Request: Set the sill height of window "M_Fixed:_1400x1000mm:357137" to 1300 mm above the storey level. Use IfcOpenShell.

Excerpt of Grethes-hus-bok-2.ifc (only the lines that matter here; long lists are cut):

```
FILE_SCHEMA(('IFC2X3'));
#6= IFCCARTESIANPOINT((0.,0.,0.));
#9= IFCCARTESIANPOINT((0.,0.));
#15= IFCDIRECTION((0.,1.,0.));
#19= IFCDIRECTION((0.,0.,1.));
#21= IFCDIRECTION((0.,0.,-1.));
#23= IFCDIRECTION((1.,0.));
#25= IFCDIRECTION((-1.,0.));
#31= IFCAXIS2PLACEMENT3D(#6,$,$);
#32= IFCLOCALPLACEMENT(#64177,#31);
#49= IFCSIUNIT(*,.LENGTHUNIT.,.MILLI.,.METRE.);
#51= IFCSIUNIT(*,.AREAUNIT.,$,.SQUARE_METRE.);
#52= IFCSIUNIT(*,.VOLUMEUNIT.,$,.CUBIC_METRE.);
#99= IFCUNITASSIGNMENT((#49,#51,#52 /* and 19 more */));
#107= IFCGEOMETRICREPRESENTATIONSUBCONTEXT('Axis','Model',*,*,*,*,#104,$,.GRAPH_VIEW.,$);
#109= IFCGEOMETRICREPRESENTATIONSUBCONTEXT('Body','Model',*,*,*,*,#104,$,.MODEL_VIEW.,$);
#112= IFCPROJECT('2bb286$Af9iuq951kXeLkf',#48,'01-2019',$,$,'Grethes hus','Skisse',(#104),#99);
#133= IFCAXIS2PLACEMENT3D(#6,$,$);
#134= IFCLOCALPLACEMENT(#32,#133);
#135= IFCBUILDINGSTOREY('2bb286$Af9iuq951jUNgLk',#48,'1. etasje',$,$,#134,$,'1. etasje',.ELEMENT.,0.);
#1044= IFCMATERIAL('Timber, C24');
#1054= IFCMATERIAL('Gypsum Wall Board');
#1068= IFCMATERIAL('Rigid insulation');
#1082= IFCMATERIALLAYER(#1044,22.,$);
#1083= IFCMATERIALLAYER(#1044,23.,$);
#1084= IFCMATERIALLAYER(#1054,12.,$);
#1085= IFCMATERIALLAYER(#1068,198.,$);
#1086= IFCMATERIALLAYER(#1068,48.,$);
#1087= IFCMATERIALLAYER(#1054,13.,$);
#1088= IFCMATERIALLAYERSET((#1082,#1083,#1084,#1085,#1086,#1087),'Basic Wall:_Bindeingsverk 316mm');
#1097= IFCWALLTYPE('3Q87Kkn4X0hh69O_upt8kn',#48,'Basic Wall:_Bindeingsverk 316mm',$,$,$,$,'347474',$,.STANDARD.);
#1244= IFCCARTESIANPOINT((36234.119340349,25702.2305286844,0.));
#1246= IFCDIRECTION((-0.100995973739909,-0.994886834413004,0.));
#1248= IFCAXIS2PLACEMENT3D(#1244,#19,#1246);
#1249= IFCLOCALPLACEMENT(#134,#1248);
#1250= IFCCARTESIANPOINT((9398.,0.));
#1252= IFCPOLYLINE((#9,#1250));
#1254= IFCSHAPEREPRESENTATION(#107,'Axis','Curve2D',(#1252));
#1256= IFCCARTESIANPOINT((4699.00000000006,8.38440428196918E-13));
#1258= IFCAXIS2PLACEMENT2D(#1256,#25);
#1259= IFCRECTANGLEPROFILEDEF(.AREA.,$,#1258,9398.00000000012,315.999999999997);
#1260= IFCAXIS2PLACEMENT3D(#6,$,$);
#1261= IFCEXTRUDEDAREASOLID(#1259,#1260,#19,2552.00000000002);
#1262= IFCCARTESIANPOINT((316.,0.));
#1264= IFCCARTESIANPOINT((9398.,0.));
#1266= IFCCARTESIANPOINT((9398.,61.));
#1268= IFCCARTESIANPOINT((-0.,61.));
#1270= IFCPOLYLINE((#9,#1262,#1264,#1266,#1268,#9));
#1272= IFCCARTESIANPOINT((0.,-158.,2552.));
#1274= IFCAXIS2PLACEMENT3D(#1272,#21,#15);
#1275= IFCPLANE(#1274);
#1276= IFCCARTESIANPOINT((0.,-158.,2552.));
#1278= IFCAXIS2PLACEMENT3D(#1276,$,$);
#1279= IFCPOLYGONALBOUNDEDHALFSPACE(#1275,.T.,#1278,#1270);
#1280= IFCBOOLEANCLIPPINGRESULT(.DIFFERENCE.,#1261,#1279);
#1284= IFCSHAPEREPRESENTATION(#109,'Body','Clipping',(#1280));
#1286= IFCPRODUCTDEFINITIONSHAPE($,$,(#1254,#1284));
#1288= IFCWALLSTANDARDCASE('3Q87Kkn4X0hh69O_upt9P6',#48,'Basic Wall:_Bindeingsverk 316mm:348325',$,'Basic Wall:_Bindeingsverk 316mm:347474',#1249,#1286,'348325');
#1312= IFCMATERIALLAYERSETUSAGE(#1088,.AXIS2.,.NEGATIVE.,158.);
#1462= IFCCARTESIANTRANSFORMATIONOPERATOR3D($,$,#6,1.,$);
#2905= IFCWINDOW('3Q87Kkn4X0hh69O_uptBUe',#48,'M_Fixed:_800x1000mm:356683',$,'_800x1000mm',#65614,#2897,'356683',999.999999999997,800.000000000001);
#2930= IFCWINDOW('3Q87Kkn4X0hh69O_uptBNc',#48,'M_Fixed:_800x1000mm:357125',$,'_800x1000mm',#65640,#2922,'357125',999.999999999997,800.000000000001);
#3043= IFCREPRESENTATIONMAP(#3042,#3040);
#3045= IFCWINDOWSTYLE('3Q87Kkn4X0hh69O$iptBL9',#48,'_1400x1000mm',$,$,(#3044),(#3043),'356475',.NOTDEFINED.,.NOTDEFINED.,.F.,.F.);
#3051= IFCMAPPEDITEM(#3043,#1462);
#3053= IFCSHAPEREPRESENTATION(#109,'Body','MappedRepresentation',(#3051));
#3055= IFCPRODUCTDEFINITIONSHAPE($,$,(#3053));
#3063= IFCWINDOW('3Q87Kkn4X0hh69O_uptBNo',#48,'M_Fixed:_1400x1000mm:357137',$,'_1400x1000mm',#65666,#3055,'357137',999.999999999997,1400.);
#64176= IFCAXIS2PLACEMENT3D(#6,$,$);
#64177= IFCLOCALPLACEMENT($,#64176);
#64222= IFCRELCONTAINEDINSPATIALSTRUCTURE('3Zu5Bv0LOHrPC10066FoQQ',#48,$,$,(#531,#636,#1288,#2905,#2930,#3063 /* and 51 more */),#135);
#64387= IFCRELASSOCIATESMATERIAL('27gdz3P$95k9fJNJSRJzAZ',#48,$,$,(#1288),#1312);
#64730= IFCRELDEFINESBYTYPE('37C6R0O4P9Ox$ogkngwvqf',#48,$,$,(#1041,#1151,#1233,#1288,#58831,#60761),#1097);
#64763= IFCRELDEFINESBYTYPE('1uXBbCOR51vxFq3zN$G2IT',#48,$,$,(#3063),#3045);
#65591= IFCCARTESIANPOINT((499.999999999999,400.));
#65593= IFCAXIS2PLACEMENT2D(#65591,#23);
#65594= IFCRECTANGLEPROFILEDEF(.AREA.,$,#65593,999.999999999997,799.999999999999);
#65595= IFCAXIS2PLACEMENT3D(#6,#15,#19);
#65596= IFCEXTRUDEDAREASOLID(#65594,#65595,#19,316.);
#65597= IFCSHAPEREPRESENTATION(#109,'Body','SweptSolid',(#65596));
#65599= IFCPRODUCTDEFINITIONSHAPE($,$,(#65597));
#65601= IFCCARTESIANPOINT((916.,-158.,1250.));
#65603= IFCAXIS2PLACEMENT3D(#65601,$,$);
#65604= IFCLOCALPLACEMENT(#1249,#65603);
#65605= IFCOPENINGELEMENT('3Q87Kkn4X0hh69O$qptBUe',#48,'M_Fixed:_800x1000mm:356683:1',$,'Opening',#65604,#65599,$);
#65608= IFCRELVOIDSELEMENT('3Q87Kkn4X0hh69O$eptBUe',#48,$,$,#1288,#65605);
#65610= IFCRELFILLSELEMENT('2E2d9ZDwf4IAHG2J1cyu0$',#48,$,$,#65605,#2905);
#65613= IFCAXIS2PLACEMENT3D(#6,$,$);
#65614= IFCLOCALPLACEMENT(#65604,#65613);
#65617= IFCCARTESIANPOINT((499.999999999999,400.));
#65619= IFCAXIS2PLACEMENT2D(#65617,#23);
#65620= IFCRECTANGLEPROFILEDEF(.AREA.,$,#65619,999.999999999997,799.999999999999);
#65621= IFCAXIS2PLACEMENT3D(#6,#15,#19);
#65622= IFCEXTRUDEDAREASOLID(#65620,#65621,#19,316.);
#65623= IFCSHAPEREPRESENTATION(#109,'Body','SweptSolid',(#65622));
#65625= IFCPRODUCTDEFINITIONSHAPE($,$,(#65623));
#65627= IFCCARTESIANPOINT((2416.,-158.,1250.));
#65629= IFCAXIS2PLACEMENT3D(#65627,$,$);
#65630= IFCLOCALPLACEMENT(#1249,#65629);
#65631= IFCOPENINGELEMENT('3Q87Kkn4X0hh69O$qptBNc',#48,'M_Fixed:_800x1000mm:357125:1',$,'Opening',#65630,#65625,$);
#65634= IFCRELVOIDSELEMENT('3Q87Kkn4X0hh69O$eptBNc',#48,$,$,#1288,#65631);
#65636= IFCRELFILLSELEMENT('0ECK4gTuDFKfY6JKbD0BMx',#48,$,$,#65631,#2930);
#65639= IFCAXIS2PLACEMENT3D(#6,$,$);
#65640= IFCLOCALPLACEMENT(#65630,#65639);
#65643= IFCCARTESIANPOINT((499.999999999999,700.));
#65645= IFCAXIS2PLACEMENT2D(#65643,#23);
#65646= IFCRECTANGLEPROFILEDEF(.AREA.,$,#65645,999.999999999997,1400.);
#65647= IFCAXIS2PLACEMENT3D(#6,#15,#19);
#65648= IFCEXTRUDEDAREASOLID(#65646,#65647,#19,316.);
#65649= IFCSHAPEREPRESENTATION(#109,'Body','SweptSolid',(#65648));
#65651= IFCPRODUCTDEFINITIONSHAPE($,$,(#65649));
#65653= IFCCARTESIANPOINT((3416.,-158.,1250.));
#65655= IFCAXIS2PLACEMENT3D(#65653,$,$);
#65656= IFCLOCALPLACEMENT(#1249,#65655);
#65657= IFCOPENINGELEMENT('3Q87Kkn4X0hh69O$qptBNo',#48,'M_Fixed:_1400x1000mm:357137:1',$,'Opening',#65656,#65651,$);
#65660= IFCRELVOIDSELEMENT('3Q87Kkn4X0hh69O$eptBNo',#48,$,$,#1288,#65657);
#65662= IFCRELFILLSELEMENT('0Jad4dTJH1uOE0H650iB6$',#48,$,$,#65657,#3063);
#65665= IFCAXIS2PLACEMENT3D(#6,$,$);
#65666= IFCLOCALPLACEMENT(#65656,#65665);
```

```python
import numpy as np
import ifcopenshell
import ifcopenshell.api.geometry
import ifcopenshell.geom
import ifcopenshell.util.element
import ifcopenshell.util.placement
import ifcopenshell.util.shape
import ifcopenshell.util.unit

model = ifcopenshell.open("Grethes-hus-bok-2.ifc")
unit_scale = ifcopenshell.util.unit.calculate_unit_scale(model)

window = model.by_guid("3Q87Kkn4X0hh69O_uptBNo")
opening = window.FillsVoids[0].RelatingOpeningElement
storey = ifcopenshell.util.element.get_container(window, ifc_class="IfcBuildingStorey")
level = ifcopenshell.util.placement.get_local_placement(storey.ObjectPlacement)[2, 3]

# The opening's origin need not be at the sill, so measure its lowest point.
shape = ifcopenshell.geom.create_shape(ifcopenshell.geom.settings(), opening)
bottom = ifcopenshell.util.shape.get_shape_bottom_elevation(shape, shape.geometry) / unit_scale
dz = level + 1300.0 - bottom

shift = np.array([0.0, 0.0, dz])
# The window is placed relative to its opening, so it follows when the opening moves.
matrix = ifcopenshell.util.placement.get_local_placement(opening.ObjectPlacement)
matrix[:3, 3] += shift
ifcopenshell.api.geometry.edit_object_placement(
    model, product=opening, matrix=matrix, is_si=False, should_transform_children=True
)

print(f"moved by {dz * unit_scale:+.3f} m")

model.write("Grethes-hus-bok-2_edited.ifc")
```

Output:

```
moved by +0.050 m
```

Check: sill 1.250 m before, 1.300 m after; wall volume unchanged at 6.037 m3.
